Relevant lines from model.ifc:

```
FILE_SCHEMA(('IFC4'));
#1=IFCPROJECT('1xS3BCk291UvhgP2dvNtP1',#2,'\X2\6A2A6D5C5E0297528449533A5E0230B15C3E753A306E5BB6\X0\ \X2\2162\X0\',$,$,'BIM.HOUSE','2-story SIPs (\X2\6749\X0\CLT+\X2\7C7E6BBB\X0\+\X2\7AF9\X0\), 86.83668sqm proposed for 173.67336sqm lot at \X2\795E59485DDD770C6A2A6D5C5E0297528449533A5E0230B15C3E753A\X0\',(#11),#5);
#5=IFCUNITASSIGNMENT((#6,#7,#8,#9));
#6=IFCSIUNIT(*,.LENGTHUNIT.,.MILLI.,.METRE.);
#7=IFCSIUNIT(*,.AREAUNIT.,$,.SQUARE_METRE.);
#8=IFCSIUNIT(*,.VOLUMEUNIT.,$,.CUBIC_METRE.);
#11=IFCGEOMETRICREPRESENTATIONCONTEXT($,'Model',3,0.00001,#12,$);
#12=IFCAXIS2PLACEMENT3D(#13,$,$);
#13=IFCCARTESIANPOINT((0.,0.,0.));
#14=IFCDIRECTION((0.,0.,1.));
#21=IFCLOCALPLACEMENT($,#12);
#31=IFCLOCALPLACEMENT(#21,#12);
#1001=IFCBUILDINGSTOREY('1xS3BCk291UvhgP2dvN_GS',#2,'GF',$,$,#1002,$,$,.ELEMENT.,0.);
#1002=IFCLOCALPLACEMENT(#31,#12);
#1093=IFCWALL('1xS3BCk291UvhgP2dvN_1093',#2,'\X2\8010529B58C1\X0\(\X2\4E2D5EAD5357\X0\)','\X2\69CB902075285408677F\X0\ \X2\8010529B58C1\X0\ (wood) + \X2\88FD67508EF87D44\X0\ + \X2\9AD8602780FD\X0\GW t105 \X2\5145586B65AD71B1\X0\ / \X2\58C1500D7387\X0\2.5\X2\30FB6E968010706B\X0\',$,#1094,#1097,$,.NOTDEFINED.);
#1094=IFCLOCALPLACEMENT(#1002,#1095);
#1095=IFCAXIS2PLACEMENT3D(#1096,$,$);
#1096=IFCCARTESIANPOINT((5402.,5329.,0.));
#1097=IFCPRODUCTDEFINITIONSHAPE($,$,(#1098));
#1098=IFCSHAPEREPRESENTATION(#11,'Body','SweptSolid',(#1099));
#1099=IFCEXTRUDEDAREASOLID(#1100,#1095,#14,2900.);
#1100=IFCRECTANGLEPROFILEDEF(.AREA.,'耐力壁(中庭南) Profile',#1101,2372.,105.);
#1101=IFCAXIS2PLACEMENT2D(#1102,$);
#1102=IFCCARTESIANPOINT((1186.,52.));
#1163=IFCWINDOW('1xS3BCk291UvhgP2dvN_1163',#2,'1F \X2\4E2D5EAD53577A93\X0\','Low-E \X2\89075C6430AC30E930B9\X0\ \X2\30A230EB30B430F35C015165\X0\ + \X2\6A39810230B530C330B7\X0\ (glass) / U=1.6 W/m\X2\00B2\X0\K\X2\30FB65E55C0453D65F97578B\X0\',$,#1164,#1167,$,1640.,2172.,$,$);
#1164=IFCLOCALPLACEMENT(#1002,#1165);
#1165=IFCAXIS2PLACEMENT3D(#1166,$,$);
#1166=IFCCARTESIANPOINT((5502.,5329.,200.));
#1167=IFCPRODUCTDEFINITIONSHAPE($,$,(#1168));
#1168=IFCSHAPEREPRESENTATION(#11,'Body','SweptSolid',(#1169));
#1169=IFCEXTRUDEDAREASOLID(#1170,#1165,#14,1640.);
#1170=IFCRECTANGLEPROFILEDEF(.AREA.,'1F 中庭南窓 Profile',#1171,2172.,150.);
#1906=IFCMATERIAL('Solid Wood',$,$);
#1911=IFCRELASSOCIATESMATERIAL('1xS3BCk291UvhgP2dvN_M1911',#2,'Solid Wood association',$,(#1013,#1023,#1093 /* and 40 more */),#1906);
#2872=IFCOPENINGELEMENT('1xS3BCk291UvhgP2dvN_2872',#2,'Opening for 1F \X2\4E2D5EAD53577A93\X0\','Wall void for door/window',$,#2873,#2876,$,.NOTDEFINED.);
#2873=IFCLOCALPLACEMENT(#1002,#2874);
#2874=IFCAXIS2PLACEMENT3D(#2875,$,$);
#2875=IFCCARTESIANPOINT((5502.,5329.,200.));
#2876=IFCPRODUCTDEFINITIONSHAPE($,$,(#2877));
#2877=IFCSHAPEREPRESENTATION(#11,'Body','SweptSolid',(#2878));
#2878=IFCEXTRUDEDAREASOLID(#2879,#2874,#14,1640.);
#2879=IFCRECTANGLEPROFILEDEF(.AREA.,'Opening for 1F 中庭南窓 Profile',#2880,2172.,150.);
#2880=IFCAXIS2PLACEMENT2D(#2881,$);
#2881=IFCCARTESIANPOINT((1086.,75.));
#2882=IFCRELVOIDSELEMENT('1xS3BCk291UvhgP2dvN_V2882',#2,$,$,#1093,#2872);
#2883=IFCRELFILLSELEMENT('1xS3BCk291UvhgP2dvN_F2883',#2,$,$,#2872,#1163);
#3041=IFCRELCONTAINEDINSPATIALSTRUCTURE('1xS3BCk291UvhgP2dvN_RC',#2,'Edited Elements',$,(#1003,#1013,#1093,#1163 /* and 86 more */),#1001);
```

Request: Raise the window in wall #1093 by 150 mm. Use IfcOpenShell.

```python
import numpy as np
import ifcopenshell
import ifcopenshell.api.geometry
import ifcopenshell.util.placement
import ifcopenshell.util.unit

model = ifcopenshell.open("model.ifc")
unit_scale = ifcopenshell.util.unit.calculate_unit_scale(model)

window = model.by_guid("1xS3BCk291UvhgP2dvN_1163")
opening = window.FillsVoids[0].RelatingOpeningElement
dz = 150.0

shift = np.array([0.0, 0.0, dz])
# The window is not placed relative to its opening, so move both.
for product in (opening, window):
    matrix = ifcopenshell.util.placement.get_local_placement(product.ObjectPlacement)
    matrix[:3, 3] += shift
    ifcopenshell.api.geometry.edit_object_placement(model, product=product, matrix=matrix, is_si=False)

print(f"moved by {dz * unit_scale:+.3f} m")

model.write("model_edited.ifc")
```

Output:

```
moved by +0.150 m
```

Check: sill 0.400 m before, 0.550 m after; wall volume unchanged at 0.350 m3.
